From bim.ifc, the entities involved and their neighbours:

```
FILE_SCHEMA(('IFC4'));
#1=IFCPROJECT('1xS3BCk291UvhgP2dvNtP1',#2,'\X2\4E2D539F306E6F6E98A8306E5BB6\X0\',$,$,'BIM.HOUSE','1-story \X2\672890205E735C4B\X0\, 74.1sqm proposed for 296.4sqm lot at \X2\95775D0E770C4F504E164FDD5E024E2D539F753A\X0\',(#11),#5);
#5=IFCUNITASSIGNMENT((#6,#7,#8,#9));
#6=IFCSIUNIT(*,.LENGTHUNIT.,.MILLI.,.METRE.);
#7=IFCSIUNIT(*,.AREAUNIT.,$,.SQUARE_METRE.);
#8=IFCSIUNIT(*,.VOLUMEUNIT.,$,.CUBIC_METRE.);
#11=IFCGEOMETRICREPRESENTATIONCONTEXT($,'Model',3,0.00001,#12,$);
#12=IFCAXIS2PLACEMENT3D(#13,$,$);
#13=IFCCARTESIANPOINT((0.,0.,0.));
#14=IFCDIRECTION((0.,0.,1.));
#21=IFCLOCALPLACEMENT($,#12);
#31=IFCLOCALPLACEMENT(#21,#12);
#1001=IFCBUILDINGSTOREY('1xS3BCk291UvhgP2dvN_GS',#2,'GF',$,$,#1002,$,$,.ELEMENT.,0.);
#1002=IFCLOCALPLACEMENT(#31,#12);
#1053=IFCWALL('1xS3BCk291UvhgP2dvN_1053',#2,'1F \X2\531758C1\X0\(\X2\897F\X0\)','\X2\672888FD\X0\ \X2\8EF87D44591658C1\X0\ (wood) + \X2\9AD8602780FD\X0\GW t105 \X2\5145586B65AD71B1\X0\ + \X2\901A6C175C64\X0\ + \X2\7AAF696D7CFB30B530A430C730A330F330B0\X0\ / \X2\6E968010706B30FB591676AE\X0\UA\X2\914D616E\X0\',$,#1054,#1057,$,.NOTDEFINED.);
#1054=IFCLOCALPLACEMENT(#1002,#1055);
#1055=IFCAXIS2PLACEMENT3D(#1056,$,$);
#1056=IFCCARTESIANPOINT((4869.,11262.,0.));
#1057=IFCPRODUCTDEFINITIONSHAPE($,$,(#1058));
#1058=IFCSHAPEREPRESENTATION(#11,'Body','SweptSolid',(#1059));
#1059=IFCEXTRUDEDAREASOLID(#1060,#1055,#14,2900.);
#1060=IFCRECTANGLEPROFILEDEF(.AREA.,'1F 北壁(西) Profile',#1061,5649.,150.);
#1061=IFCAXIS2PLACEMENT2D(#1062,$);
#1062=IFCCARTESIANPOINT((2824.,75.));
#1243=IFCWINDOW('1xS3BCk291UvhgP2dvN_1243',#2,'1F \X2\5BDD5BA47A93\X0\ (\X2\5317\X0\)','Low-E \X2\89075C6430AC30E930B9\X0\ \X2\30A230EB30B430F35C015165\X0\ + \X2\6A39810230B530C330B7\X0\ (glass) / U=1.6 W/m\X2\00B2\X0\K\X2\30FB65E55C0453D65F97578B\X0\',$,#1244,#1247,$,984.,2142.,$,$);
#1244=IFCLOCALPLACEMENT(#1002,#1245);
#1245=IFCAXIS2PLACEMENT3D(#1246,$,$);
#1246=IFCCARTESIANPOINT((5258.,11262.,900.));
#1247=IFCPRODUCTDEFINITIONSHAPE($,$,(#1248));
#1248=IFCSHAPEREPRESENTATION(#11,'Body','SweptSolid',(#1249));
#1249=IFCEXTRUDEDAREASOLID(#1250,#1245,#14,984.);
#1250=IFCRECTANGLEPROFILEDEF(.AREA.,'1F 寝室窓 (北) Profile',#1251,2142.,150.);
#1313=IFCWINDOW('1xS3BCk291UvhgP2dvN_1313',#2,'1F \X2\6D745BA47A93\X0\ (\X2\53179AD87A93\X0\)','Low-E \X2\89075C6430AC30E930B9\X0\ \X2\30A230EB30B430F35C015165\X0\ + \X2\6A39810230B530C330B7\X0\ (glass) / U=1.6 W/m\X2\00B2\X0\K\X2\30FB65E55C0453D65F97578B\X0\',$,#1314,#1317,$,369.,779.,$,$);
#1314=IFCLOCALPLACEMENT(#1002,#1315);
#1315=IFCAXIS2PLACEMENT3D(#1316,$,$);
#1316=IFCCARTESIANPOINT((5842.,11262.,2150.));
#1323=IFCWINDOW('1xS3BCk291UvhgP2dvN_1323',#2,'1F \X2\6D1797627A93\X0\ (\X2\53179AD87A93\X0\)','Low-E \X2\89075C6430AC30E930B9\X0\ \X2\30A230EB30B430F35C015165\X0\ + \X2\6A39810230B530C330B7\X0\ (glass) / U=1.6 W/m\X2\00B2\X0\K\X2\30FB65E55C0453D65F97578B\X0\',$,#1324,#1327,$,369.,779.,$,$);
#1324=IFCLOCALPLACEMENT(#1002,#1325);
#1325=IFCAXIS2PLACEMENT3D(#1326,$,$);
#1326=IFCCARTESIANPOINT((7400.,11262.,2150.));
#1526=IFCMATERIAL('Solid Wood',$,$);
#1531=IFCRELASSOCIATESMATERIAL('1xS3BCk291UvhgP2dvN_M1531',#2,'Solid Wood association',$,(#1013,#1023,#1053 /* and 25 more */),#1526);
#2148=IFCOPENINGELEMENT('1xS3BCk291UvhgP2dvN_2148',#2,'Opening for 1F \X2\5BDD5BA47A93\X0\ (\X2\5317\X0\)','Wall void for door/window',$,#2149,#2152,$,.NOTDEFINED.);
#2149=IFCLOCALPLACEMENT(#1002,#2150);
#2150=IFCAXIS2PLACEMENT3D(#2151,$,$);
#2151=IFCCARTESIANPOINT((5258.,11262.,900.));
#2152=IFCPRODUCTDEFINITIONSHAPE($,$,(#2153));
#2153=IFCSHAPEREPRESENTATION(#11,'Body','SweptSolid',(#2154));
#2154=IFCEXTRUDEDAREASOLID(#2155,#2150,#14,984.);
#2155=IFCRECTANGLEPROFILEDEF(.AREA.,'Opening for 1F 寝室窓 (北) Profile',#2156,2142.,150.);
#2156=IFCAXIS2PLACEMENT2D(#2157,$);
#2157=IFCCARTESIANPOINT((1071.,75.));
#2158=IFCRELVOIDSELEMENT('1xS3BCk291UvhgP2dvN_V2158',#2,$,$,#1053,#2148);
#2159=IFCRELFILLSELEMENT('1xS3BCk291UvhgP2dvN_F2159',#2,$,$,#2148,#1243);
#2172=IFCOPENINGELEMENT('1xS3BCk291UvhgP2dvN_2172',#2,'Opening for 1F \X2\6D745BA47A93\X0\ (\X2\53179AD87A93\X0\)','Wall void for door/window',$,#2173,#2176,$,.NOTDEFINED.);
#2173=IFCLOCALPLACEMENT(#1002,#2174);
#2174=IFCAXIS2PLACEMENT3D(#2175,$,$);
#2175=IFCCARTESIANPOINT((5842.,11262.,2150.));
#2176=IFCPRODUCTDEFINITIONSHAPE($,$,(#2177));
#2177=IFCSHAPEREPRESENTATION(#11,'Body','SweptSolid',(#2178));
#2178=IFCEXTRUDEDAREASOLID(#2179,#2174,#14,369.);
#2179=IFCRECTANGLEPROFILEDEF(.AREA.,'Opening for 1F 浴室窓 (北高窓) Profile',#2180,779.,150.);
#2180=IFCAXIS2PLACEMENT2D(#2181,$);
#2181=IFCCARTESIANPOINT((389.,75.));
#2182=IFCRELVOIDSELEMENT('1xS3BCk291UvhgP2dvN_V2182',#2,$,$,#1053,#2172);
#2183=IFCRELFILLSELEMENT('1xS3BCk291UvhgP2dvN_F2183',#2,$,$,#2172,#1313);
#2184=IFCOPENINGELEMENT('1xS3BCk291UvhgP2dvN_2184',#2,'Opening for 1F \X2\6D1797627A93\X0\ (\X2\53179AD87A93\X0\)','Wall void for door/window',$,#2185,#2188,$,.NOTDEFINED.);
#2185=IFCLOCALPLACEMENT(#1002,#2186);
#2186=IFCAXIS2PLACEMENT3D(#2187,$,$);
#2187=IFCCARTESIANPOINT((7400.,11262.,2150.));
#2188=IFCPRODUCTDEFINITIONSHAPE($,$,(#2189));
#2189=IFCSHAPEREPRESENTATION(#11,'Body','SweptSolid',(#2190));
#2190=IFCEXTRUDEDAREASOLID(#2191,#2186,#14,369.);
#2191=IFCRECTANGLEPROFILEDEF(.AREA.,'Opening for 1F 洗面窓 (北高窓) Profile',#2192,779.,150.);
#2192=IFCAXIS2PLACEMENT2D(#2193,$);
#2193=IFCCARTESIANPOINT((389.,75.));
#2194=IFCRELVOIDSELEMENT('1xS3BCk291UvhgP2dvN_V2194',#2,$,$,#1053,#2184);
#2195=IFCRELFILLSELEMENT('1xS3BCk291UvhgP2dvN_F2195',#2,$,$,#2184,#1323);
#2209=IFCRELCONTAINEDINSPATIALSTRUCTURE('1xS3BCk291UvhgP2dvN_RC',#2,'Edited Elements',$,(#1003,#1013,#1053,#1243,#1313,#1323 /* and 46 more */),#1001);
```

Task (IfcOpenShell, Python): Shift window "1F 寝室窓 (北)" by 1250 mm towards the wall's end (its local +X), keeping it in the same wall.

```python
import ifcopenshell
import ifcopenshell.api.geometry
import ifcopenshell.util.placement

model = ifcopenshell.open("bim.ifc")

window = model.by_guid("1xS3BCk291UvhgP2dvN_1243")
opening = window.FillsVoids[0].RelatingOpeningElement
wall = opening.VoidsElements[0].RelatingBuildingElement

wall_matrix = ifcopenshell.util.placement.get_local_placement(wall.ObjectPlacement)
shift = wall_matrix[:3, 0] * 1250.0
before = ifcopenshell.util.placement.get_local_placement(window.ObjectPlacement)[:3, 3].copy()

# The window is not placed relative to its opening, so move both.
for product in (opening, window):
    matrix = ifcopenshell.util.placement.get_local_placement(product.ObjectPlacement)
    matrix[:3, 3] += shift
    ifcopenshell.api.geometry.edit_object_placement(model, product=product, matrix=matrix, is_si=False)

after = ifcopenshell.util.placement.get_local_placement(window.ObjectPlacement)[:3, 3]
print("window moved by", (after - before).round(3) + 0.0)

model.write("bim_edited.ifc")
```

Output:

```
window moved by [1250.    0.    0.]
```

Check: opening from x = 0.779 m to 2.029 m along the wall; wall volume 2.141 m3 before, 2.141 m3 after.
